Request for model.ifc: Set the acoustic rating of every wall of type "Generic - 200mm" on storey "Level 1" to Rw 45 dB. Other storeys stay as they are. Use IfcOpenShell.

First a look at what the model holds.

```python
import ifcopenshell
import ifcopenshell.util.element

model = ifcopenshell.open("model.ifc")
print(model.schema)
storey = next(s for s in model.by_type("IfcBuildingStorey") if s.Name == "Level 1")
walls = [e for e in ifcopenshell.util.element.get_decomposition(storey) if e.is_a("IfcWall")]
seen = {}
for e in walls:
    element_type = ifcopenshell.util.element.get_type(e)
    key = (element_type.Name if element_type != e and element_type else None, ifcopenshell.util.element.get_pset(e, "Pset_WallCommon", "AcousticRating"))
    seen[key] = seen.get(key, 0) + 1
for (name, value), count in sorted(seen.items(), key=str):
    print(count, "x", name, "|", value)
```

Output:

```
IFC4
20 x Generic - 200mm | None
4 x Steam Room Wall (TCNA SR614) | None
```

```python
import ifcopenshell
import ifcopenshell.api.pset
import ifcopenshell.util.element

model = ifcopenshell.open("model.ifc")

storey = next(s for s in model.by_type("IfcBuildingStorey") if s.Name == "Level 1")
walls = [e for e in ifcopenshell.util.element.get_decomposition(storey) if e.is_a("IfcWall")]

count = 0
for e in walls:
    element_type = ifcopenshell.util.element.get_type(e)
    if element_type in (None, e) or element_type.Name != "Generic - 200mm":
        continue
    # add_pset returns the element's existing set when there is one.
    pset = ifcopenshell.api.pset.add_pset(model, product=e, name="Pset_WallCommon")
    ifcopenshell.api.pset.edit_pset(model, pset=pset, properties={"AcousticRating": "Rw 45 dB"})
    count += 1

print(count, "walls updated")

model.write("model_edited.ifc")
```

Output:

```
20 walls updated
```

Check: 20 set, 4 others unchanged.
